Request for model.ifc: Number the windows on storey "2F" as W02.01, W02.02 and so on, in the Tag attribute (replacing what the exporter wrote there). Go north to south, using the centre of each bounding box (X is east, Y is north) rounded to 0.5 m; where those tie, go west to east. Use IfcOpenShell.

First a look at what the model holds.

```python
import ifcopenshell
import ifcopenshell.util.element
import ifcopenshell.util.placement

model = ifcopenshell.open("model.ifc")
print(model.schema)
storey = next(s for s in model.by_type("IfcBuildingStorey") if s.Name == "2F")
windows = [e for e in ifcopenshell.util.element.get_decomposition(storey) if e.is_a("IfcWindow")]
for e in sorted(windows, key=lambda e: e.id()):
    origin = ifcopenshell.util.placement.get_local_placement(e.ObjectPlacement)[:3, 3]
    print(e.id(), e.Tag, e.Name, origin.round(2) + 0.0, sep=" | ")
```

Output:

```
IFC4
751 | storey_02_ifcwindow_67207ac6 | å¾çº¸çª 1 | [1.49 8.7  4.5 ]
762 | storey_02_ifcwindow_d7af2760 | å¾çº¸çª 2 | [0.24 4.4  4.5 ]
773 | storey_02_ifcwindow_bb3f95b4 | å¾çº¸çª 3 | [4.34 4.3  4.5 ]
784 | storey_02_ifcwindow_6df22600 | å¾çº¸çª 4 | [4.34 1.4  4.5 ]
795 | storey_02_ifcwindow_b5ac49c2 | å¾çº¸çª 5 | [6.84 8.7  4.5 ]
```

```python
import ifcopenshell
import ifcopenshell.geom
import ifcopenshell.util.element
import ifcopenshell.util.shape

model = ifcopenshell.open("model.ifc")
settings = ifcopenshell.geom.settings()
settings.set("use-world-coords", True)


def centre(element):
    shape = ifcopenshell.geom.create_shape(settings, element)
    return ifcopenshell.util.shape.get_bbox_centroid(shape.geometry)


storey = next(s for s in model.by_type("IfcBuildingStorey") if s.Name == "2F")
windows = [e for e in ifcopenshell.util.element.get_decomposition(storey) if e.is_a("IfcWindow")]

# Insertion points can sit at a corner or the storey origin, so sort by the geometry (in metres).
centres = {e: centre(e) for e in windows}
windows.sort(key=lambda e: (-round(centres[e][1] / 0.5), centres[e][0]))

for i, e in enumerate(windows, start=1):
    number = f"W02.{i:02d}"
    e.Tag = number
    print(e.id(), number)

model.write("model_v2.ifc")
```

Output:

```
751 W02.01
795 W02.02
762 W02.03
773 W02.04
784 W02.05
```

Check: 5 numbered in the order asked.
